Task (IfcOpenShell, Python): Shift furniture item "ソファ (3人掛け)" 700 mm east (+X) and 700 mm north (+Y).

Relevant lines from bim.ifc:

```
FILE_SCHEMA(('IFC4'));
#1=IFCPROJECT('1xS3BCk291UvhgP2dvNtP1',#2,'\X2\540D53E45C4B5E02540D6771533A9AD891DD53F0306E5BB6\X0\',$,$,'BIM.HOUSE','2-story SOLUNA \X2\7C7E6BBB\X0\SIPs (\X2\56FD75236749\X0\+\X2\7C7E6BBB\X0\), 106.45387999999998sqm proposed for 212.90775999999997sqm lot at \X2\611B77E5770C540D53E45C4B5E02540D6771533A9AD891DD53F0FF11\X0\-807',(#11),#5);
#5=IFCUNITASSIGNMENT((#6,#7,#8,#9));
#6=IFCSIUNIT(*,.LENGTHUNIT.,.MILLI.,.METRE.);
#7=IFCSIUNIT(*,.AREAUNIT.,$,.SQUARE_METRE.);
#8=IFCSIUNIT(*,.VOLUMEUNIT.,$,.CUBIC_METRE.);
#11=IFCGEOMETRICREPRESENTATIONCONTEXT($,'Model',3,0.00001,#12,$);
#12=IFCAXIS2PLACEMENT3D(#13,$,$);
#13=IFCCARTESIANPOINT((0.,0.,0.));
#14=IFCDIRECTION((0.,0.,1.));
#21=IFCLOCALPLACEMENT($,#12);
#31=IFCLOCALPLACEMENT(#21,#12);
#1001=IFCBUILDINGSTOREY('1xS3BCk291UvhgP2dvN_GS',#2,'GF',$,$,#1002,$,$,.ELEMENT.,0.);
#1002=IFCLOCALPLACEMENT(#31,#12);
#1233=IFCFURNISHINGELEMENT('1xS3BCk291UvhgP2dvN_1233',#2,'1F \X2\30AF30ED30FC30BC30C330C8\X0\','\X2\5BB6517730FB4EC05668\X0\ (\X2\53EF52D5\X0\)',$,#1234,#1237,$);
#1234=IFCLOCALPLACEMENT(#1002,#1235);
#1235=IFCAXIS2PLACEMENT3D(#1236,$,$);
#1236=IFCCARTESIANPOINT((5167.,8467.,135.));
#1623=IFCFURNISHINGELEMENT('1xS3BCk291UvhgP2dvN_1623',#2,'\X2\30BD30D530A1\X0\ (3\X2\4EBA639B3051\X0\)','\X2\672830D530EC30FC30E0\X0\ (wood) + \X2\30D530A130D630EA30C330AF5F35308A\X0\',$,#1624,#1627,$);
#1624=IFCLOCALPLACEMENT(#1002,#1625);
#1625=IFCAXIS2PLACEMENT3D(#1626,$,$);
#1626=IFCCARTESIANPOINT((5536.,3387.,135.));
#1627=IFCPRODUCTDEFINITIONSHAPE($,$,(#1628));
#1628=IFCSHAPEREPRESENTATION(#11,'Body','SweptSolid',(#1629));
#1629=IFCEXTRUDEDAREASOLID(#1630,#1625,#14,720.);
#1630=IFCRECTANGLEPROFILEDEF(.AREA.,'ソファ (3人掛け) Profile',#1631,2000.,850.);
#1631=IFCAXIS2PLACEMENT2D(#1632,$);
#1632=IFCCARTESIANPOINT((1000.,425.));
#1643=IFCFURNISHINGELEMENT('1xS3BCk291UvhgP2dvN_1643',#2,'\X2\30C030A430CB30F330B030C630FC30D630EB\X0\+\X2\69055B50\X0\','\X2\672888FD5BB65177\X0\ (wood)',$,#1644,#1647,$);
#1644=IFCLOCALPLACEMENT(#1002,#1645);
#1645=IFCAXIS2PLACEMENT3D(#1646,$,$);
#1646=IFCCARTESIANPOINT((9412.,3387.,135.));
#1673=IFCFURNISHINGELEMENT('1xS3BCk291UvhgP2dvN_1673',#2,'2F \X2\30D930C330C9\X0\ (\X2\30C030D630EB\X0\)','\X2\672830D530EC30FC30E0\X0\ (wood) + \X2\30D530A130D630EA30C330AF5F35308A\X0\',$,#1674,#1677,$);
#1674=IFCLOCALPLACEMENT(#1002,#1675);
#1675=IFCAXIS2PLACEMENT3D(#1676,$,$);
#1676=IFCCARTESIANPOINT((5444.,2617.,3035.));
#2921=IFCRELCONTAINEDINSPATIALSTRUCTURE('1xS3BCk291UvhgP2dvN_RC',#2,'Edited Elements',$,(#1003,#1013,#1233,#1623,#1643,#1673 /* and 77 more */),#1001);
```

```python
import ifcopenshell
import ifcopenshell.api.geometry
import ifcopenshell.util.placement
import ifcopenshell.util.unit

model = ifcopenshell.open("bim.ifc")
unit_scale = ifcopenshell.util.unit.calculate_unit_scale(model)

item = model.by_guid("1xS3BCk291UvhgP2dvN_1623")
matrix = ifcopenshell.util.placement.get_local_placement(item.ObjectPlacement)
matrix[0, 3] += 0.7 / unit_scale
matrix[1, 3] += 0.7 / unit_scale
ifcopenshell.api.geometry.edit_object_placement(model, product=item, matrix=matrix, is_si=False)

print(ifcopenshell.util.placement.get_local_placement(item.ObjectPlacement).round(3) + 0.0)

model.write("bim_updated.ifc")
```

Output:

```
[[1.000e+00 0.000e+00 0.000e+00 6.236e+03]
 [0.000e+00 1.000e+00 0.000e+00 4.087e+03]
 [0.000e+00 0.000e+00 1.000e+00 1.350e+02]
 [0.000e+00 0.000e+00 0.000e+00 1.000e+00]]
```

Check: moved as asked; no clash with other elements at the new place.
